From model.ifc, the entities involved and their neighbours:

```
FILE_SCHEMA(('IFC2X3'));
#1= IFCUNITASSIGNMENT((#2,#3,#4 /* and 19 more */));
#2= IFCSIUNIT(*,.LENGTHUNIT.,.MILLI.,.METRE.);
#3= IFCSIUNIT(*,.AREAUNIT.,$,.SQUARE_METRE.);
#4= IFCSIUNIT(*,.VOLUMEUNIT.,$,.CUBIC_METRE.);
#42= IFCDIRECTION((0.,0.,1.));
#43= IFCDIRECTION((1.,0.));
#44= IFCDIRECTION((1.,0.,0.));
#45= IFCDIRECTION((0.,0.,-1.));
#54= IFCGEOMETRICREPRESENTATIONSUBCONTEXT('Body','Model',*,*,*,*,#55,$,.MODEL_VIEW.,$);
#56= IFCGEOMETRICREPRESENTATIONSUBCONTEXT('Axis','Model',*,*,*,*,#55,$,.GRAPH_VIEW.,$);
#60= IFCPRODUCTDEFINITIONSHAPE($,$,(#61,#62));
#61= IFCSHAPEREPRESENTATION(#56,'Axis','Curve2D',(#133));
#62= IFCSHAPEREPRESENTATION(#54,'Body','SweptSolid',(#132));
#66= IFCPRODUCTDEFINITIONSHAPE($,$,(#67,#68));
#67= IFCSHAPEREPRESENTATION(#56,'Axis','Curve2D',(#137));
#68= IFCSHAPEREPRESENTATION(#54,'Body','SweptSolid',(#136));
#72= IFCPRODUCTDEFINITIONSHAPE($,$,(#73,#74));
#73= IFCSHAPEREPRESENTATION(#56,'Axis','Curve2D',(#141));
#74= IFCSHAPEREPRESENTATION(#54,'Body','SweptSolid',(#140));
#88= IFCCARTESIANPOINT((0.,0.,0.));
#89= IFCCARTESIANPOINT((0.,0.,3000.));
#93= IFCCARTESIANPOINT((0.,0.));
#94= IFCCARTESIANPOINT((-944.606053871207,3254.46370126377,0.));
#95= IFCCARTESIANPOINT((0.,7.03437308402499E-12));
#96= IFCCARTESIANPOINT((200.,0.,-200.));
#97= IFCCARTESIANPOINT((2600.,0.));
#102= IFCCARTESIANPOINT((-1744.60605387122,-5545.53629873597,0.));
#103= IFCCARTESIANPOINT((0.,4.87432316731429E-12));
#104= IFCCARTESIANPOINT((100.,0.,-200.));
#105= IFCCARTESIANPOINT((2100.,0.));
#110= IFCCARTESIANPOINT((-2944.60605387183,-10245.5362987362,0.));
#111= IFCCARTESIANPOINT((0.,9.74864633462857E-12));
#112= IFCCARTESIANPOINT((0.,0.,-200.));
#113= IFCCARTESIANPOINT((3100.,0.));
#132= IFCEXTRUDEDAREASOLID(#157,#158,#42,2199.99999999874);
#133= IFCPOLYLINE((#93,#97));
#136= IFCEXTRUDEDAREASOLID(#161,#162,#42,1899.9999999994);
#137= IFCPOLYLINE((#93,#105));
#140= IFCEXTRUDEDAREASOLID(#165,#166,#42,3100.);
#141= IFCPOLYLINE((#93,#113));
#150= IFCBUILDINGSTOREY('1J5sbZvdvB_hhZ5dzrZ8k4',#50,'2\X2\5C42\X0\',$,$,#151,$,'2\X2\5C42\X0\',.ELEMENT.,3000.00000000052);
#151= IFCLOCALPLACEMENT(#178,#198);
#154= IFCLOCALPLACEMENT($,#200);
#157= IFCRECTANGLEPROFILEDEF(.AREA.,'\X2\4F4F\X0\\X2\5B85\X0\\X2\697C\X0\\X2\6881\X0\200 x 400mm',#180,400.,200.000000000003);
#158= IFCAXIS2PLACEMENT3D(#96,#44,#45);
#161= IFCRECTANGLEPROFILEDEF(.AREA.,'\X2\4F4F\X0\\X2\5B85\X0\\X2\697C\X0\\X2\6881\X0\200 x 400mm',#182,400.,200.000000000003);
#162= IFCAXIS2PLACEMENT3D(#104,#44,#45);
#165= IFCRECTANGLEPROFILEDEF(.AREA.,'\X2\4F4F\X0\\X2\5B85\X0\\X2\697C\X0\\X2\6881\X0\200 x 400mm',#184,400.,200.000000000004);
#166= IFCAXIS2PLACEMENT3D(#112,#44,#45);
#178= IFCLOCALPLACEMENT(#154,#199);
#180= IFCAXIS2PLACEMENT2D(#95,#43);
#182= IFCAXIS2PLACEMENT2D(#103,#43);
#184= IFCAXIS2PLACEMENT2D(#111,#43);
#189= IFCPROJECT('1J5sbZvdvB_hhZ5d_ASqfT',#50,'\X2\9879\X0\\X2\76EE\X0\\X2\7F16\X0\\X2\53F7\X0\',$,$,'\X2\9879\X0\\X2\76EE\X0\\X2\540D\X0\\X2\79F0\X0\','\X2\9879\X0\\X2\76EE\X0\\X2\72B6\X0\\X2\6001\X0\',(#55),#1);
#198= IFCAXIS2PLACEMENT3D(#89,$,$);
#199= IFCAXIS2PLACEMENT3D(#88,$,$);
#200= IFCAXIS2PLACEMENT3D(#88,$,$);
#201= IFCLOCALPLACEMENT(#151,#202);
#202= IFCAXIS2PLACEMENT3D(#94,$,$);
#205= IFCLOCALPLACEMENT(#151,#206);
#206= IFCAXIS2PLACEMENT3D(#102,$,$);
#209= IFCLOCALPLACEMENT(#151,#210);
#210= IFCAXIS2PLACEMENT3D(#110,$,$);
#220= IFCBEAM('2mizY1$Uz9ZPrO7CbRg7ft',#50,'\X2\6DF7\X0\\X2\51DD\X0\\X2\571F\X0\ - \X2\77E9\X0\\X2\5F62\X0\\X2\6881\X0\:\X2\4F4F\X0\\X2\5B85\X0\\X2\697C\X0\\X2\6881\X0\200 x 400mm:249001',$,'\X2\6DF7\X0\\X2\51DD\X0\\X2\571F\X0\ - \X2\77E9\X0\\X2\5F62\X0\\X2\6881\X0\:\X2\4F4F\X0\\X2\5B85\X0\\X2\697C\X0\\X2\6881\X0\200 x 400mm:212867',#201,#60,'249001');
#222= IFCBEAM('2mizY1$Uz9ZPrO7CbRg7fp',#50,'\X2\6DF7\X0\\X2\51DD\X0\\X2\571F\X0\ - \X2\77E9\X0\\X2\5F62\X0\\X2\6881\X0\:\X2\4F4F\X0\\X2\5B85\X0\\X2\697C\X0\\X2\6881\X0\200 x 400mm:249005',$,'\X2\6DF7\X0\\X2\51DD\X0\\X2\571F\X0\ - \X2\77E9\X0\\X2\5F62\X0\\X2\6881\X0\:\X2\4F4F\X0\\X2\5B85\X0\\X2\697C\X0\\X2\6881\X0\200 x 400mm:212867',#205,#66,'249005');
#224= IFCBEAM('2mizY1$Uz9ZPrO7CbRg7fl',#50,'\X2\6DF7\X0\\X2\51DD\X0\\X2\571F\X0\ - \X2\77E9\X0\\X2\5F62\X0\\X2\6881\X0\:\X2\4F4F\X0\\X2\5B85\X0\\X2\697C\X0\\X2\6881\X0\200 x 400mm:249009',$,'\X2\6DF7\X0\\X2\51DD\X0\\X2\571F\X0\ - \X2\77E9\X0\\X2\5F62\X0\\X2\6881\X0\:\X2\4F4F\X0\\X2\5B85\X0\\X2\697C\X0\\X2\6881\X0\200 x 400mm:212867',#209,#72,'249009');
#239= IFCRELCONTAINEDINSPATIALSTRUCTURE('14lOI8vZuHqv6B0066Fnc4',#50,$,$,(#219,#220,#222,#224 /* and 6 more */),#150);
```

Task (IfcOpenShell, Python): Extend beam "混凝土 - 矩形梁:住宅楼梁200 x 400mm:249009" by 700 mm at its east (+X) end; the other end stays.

```python
import numpy as np
import ifcopenshell
import ifcopenshell.util.representation

model = ifcopenshell.open("model.ifc")

member = model.by_guid("2mizY1$Uz9ZPrO7CbRg7fl")
change = 700.0

# The extrusion runs towards the end named, so only its depth changes.
body = ifcopenshell.util.representation.get_representation(member, "Model", "Body")
solid = body.Items[0]
old_length = solid.Depth
solid.Depth += change

# Move the axis end point with it.
axis = next(r for r in member.Representation.Representations if r.RepresentationIdentifier == "Axis").Items[0]
start, end = (np.array(p.Coordinates) for p in axis.Points)
end = end + (end - start) / np.linalg.norm(end - start) * change
point = model.createIfcCartesianPoint(end.tolist())
axis.Points = [axis.Points[0], point]

print(f"length {old_length:g} -> {solid.Depth:g}")

model.write("model_rev.ifc")
```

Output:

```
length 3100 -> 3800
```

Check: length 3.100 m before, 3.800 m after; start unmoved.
